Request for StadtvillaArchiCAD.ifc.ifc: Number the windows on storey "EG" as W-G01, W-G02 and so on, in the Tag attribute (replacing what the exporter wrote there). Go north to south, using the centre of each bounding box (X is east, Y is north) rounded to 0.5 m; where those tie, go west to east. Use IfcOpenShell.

First a look at what the model holds.

```python
import ifcopenshell
import ifcopenshell.util.element
import ifcopenshell.util.placement

model = ifcopenshell.open("StadtvillaArchiCAD.ifc.ifc")
print(model.schema)
storey = next(s for s in model.by_type("IfcBuildingStorey") if s.Name == "EG")
windows = [e for e in ifcopenshell.util.element.get_decomposition(storey) if e.is_a("IfcWindow")]
for e in sorted(windows, key=lambda e: e.id()):
    origin = ifcopenshell.util.placement.get_local_placement(e.ObjectPlacement)[:3, 3]
    print(e.id(), e.Tag, e.Name, origin.round(2) + 0.0, sep=" | ")
```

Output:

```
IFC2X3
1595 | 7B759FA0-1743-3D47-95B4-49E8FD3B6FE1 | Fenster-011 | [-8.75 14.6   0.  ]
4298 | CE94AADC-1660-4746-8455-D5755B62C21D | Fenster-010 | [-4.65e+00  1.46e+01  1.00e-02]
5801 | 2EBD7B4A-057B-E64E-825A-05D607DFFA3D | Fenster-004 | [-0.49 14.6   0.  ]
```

```python
import ifcopenshell
import ifcopenshell.geom
import ifcopenshell.util.element
import ifcopenshell.util.shape

model = ifcopenshell.open("StadtvillaArchiCAD.ifc.ifc")
settings = ifcopenshell.geom.settings()
settings.set("use-world-coords", True)


def centre(element):
    shape = ifcopenshell.geom.create_shape(settings, element)
    return ifcopenshell.util.shape.get_bbox_centroid(shape.geometry)


storey = next(s for s in model.by_type("IfcBuildingStorey") if s.Name == "EG")
windows = [e for e in ifcopenshell.util.element.get_decomposition(storey) if e.is_a("IfcWindow")]

# Insertion points can sit at a corner or the storey origin, so sort by the geometry (in metres).
centres = {e: centre(e) for e in windows}
windows.sort(key=lambda e: (-round(centres[e][1] / 0.5), centres[e][0]))

for i, e in enumerate(windows, start=1):
    number = f"W-G{i:02d}"
    e.Tag = number
    print(e.id(), number)

model.write("StadtvillaArchiCAD.ifc-out.ifc")
```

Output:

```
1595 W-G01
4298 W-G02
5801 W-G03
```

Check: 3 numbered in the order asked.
